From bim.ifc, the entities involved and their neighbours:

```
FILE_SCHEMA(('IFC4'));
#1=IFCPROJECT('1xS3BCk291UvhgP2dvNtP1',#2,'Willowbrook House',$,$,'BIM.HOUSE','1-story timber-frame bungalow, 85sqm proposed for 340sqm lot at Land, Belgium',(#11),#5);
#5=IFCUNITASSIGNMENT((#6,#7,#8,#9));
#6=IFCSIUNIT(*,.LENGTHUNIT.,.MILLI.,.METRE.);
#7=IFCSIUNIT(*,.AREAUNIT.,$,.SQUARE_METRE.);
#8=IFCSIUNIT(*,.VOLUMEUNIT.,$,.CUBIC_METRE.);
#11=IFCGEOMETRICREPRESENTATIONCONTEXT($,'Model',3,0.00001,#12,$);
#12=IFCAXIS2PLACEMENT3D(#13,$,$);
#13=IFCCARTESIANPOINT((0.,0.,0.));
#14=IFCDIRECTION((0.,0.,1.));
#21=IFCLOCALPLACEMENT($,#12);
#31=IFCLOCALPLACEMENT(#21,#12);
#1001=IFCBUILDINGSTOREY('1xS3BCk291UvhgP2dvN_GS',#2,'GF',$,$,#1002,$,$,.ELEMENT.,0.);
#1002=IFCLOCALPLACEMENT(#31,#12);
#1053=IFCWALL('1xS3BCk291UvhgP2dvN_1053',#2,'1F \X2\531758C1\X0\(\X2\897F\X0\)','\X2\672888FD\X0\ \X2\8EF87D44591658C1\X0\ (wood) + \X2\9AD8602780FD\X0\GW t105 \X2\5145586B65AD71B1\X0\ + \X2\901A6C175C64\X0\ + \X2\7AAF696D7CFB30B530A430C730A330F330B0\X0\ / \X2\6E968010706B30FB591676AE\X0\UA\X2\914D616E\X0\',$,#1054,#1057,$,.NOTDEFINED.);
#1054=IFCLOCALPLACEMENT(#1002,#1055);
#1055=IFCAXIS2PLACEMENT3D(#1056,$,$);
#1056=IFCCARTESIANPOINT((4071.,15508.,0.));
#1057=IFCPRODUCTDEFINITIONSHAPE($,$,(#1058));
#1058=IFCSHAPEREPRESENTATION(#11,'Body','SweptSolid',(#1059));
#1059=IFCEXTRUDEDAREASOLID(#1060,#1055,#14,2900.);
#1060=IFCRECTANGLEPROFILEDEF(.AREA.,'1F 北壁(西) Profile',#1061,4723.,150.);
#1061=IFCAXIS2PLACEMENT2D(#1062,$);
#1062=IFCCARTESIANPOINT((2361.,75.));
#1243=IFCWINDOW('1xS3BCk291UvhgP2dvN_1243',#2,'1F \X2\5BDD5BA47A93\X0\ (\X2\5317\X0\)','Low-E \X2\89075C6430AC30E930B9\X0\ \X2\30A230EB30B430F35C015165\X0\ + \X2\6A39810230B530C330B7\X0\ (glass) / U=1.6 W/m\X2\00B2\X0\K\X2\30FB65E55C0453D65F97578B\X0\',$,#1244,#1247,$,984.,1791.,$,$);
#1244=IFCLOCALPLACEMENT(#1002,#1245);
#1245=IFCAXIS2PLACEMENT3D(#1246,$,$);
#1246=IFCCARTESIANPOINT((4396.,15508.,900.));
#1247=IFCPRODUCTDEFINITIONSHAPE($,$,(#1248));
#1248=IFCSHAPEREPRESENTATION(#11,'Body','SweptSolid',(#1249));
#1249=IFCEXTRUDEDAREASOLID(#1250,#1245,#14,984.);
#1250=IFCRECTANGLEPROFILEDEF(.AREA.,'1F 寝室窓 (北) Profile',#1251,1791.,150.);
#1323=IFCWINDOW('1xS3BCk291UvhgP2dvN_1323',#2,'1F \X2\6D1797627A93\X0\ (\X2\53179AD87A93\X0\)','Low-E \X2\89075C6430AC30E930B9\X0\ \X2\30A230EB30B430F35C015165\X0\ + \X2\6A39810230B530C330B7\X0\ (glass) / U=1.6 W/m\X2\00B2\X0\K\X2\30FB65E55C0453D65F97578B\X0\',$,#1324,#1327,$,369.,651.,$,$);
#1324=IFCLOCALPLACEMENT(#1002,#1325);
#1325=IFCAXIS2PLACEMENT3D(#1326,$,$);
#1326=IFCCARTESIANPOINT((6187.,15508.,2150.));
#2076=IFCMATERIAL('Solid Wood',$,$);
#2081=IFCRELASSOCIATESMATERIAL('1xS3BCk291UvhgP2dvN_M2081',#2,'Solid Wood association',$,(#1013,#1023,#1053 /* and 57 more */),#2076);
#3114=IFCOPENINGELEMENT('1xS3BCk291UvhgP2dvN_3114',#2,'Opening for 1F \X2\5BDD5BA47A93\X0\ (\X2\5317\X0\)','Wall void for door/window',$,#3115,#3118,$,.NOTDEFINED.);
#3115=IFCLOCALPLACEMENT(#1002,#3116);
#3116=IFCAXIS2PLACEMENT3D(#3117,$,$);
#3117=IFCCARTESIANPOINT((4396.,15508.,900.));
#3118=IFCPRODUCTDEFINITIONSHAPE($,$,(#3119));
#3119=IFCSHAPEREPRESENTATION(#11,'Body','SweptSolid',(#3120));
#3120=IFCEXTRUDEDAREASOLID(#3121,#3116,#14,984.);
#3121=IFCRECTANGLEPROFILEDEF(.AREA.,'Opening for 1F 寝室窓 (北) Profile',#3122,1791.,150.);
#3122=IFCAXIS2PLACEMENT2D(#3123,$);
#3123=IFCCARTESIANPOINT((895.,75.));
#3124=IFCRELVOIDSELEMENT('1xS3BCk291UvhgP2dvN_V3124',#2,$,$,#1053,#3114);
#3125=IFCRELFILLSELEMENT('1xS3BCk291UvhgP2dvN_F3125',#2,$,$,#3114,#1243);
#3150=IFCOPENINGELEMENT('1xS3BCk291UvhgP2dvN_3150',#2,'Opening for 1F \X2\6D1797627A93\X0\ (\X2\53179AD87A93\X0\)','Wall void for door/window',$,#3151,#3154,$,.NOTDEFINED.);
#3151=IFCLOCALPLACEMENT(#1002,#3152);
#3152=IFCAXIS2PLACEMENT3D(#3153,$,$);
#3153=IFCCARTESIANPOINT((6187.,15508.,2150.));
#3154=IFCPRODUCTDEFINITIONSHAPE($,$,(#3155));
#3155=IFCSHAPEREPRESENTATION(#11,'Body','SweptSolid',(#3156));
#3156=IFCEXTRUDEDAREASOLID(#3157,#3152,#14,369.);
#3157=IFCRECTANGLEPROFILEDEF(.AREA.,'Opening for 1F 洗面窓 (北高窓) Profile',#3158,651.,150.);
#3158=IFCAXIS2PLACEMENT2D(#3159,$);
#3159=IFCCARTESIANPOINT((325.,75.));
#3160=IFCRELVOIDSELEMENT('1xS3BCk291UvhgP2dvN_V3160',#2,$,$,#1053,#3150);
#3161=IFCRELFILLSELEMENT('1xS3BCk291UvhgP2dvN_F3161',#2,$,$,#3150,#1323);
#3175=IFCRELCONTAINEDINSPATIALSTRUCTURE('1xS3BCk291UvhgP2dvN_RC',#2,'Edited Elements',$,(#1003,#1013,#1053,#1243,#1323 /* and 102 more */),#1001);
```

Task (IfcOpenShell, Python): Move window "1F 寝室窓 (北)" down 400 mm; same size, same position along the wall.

```python
import numpy as np
import ifcopenshell
import ifcopenshell.api.geometry
import ifcopenshell.util.placement
import ifcopenshell.util.unit

model = ifcopenshell.open("bim.ifc")
unit_scale = ifcopenshell.util.unit.calculate_unit_scale(model)

window = model.by_guid("1xS3BCk291UvhgP2dvN_1243")
opening = window.FillsVoids[0].RelatingOpeningElement
dz = -0.4 / unit_scale

shift = np.array([0.0, 0.0, dz])
# The window is not placed relative to its opening, so move both.
for product in (opening, window):
    matrix = ifcopenshell.util.placement.get_local_placement(product.ObjectPlacement)
    matrix[:3, 3] += shift
    ifcopenshell.api.geometry.edit_object_placement(model, product=product, matrix=matrix, is_si=False)

print(f"moved by {dz * unit_scale:+.3f} m")

model.write("bim_updated.ifc")
```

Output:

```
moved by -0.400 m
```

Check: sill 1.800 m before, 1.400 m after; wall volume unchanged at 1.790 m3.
